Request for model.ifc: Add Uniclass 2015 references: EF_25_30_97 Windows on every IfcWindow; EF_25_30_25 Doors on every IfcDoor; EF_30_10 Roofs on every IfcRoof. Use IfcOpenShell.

First a look at what the model holds.

```python
import ifcopenshell

model = ifcopenshell.open("model.ifc")
print(model.schema)
print("classifications:", [c.Name for c in model.by_type("IfcClassification")])
for ifc_class in ("IfcDoor", "IfcRoof", "IfcStair", "IfcWall", "IfcWindow"):
    print(ifc_class, len(model.by_type(ifc_class)))
```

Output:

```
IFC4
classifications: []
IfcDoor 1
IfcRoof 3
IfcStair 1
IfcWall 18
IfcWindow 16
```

```python
import ifcopenshell
import ifcopenshell.api.classification

model = ifcopenshell.open("model.ifc")

system = ifcopenshell.api.classification.add_classification(model, classification="Uniclass 2015")

codes = {
    "IfcWindow": ("EF_25_30_97", "Windows"),
    "IfcDoor": ("EF_25_30_25", "Doors"),
    "IfcRoof": ("EF_30_10", "Roofs"),
}
for ifc_class, (code, name) in codes.items():
    products = model.by_type(ifc_class)
    ifcopenshell.api.classification.add_reference(
        model, products=products, classification=system, identification=code, name=name
    )
    print(code, len(products))

model.write("model_edited.ifc")
```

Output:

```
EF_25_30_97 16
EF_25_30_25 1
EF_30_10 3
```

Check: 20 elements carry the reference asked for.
